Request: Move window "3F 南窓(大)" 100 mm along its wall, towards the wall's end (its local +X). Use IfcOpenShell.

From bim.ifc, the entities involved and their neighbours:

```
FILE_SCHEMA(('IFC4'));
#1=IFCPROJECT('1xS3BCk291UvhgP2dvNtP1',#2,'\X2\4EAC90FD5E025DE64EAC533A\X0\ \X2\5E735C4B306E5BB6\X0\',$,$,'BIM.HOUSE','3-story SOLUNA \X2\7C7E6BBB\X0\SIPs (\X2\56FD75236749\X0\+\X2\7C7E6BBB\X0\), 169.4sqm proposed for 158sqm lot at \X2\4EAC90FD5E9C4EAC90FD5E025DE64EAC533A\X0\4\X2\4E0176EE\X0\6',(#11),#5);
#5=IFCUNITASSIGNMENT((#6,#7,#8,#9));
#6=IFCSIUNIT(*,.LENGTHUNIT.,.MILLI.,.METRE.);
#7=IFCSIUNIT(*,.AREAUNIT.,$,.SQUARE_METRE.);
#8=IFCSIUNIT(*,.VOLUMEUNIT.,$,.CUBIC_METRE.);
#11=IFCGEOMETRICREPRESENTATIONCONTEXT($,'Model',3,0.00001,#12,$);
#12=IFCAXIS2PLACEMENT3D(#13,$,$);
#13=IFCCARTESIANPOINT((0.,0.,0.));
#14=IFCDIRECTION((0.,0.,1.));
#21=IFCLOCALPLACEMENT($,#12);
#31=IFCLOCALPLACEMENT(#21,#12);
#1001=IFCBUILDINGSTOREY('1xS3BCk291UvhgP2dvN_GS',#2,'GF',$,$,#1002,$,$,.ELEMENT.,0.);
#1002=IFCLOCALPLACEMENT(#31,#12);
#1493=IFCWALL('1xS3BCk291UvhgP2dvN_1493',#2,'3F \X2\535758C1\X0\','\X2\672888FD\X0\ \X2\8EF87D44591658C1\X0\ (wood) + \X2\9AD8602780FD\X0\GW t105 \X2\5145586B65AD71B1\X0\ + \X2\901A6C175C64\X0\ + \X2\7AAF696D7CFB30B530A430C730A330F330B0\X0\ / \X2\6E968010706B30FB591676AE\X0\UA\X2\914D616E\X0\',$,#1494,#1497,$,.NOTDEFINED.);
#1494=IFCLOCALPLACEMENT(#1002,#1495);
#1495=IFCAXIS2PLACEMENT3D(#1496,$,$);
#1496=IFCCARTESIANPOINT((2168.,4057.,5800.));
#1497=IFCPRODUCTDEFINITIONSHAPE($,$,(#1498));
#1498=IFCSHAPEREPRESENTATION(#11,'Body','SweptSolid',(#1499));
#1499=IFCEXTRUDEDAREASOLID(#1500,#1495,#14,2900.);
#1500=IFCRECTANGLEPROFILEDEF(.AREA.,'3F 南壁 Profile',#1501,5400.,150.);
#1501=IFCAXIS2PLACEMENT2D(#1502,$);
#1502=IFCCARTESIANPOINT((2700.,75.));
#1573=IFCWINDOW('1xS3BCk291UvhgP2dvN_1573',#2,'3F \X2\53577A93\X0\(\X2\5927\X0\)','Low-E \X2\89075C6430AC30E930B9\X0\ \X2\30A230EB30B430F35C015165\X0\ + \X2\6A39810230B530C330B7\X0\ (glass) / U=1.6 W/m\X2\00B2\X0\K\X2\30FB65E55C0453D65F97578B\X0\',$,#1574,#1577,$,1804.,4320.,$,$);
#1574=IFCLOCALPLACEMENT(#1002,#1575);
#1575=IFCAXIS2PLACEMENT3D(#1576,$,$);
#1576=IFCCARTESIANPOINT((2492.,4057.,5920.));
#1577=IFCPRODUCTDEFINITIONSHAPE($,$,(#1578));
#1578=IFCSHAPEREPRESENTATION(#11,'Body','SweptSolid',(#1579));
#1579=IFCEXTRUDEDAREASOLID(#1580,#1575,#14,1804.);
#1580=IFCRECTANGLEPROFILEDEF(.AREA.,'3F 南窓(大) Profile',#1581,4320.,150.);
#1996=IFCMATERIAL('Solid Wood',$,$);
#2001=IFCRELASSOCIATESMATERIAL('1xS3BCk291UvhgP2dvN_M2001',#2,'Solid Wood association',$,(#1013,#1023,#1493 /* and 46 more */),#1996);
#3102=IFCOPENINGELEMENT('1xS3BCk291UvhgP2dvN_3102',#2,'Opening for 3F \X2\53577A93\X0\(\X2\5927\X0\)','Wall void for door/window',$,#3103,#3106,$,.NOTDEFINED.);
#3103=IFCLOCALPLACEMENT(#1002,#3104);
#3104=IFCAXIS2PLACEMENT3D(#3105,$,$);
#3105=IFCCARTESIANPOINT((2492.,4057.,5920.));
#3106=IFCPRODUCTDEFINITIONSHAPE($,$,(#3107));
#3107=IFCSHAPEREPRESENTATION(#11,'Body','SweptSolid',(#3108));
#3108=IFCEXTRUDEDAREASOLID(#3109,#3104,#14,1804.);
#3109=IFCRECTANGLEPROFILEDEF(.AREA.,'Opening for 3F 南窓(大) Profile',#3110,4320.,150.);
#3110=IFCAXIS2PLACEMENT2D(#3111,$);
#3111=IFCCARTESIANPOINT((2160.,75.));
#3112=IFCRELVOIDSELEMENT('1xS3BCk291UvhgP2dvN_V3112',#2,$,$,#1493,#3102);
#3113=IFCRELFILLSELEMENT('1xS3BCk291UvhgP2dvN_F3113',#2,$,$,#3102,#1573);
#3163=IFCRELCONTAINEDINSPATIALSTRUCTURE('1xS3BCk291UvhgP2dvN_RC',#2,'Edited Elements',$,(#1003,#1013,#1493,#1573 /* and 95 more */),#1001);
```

```python
import ifcopenshell
import ifcopenshell.api.geometry
import ifcopenshell.util.placement

model = ifcopenshell.open("bim.ifc")

window = model.by_id(1573)
opening = window.FillsVoids[0].RelatingOpeningElement
wall = opening.VoidsElements[0].RelatingBuildingElement

wall_matrix = ifcopenshell.util.placement.get_local_placement(wall.ObjectPlacement)
shift = wall_matrix[:3, 0] * 100.0
before = ifcopenshell.util.placement.get_local_placement(window.ObjectPlacement)[:3, 3].copy()

# The window is not placed relative to its opening, so move both.
for product in (opening, window):
    matrix = ifcopenshell.util.placement.get_local_placement(product.ObjectPlacement)
    matrix[:3, 3] += shift
    ifcopenshell.api.geometry.edit_object_placement(model, product=product, matrix=matrix, is_si=False)

after = ifcopenshell.util.placement.get_local_placement(window.ObjectPlacement)[:3, 3]
print("window moved by", (after - before).round(3) + 0.0)

model.write("bim_rev.ifc")
```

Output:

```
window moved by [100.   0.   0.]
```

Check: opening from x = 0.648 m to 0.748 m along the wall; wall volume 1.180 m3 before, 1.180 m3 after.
